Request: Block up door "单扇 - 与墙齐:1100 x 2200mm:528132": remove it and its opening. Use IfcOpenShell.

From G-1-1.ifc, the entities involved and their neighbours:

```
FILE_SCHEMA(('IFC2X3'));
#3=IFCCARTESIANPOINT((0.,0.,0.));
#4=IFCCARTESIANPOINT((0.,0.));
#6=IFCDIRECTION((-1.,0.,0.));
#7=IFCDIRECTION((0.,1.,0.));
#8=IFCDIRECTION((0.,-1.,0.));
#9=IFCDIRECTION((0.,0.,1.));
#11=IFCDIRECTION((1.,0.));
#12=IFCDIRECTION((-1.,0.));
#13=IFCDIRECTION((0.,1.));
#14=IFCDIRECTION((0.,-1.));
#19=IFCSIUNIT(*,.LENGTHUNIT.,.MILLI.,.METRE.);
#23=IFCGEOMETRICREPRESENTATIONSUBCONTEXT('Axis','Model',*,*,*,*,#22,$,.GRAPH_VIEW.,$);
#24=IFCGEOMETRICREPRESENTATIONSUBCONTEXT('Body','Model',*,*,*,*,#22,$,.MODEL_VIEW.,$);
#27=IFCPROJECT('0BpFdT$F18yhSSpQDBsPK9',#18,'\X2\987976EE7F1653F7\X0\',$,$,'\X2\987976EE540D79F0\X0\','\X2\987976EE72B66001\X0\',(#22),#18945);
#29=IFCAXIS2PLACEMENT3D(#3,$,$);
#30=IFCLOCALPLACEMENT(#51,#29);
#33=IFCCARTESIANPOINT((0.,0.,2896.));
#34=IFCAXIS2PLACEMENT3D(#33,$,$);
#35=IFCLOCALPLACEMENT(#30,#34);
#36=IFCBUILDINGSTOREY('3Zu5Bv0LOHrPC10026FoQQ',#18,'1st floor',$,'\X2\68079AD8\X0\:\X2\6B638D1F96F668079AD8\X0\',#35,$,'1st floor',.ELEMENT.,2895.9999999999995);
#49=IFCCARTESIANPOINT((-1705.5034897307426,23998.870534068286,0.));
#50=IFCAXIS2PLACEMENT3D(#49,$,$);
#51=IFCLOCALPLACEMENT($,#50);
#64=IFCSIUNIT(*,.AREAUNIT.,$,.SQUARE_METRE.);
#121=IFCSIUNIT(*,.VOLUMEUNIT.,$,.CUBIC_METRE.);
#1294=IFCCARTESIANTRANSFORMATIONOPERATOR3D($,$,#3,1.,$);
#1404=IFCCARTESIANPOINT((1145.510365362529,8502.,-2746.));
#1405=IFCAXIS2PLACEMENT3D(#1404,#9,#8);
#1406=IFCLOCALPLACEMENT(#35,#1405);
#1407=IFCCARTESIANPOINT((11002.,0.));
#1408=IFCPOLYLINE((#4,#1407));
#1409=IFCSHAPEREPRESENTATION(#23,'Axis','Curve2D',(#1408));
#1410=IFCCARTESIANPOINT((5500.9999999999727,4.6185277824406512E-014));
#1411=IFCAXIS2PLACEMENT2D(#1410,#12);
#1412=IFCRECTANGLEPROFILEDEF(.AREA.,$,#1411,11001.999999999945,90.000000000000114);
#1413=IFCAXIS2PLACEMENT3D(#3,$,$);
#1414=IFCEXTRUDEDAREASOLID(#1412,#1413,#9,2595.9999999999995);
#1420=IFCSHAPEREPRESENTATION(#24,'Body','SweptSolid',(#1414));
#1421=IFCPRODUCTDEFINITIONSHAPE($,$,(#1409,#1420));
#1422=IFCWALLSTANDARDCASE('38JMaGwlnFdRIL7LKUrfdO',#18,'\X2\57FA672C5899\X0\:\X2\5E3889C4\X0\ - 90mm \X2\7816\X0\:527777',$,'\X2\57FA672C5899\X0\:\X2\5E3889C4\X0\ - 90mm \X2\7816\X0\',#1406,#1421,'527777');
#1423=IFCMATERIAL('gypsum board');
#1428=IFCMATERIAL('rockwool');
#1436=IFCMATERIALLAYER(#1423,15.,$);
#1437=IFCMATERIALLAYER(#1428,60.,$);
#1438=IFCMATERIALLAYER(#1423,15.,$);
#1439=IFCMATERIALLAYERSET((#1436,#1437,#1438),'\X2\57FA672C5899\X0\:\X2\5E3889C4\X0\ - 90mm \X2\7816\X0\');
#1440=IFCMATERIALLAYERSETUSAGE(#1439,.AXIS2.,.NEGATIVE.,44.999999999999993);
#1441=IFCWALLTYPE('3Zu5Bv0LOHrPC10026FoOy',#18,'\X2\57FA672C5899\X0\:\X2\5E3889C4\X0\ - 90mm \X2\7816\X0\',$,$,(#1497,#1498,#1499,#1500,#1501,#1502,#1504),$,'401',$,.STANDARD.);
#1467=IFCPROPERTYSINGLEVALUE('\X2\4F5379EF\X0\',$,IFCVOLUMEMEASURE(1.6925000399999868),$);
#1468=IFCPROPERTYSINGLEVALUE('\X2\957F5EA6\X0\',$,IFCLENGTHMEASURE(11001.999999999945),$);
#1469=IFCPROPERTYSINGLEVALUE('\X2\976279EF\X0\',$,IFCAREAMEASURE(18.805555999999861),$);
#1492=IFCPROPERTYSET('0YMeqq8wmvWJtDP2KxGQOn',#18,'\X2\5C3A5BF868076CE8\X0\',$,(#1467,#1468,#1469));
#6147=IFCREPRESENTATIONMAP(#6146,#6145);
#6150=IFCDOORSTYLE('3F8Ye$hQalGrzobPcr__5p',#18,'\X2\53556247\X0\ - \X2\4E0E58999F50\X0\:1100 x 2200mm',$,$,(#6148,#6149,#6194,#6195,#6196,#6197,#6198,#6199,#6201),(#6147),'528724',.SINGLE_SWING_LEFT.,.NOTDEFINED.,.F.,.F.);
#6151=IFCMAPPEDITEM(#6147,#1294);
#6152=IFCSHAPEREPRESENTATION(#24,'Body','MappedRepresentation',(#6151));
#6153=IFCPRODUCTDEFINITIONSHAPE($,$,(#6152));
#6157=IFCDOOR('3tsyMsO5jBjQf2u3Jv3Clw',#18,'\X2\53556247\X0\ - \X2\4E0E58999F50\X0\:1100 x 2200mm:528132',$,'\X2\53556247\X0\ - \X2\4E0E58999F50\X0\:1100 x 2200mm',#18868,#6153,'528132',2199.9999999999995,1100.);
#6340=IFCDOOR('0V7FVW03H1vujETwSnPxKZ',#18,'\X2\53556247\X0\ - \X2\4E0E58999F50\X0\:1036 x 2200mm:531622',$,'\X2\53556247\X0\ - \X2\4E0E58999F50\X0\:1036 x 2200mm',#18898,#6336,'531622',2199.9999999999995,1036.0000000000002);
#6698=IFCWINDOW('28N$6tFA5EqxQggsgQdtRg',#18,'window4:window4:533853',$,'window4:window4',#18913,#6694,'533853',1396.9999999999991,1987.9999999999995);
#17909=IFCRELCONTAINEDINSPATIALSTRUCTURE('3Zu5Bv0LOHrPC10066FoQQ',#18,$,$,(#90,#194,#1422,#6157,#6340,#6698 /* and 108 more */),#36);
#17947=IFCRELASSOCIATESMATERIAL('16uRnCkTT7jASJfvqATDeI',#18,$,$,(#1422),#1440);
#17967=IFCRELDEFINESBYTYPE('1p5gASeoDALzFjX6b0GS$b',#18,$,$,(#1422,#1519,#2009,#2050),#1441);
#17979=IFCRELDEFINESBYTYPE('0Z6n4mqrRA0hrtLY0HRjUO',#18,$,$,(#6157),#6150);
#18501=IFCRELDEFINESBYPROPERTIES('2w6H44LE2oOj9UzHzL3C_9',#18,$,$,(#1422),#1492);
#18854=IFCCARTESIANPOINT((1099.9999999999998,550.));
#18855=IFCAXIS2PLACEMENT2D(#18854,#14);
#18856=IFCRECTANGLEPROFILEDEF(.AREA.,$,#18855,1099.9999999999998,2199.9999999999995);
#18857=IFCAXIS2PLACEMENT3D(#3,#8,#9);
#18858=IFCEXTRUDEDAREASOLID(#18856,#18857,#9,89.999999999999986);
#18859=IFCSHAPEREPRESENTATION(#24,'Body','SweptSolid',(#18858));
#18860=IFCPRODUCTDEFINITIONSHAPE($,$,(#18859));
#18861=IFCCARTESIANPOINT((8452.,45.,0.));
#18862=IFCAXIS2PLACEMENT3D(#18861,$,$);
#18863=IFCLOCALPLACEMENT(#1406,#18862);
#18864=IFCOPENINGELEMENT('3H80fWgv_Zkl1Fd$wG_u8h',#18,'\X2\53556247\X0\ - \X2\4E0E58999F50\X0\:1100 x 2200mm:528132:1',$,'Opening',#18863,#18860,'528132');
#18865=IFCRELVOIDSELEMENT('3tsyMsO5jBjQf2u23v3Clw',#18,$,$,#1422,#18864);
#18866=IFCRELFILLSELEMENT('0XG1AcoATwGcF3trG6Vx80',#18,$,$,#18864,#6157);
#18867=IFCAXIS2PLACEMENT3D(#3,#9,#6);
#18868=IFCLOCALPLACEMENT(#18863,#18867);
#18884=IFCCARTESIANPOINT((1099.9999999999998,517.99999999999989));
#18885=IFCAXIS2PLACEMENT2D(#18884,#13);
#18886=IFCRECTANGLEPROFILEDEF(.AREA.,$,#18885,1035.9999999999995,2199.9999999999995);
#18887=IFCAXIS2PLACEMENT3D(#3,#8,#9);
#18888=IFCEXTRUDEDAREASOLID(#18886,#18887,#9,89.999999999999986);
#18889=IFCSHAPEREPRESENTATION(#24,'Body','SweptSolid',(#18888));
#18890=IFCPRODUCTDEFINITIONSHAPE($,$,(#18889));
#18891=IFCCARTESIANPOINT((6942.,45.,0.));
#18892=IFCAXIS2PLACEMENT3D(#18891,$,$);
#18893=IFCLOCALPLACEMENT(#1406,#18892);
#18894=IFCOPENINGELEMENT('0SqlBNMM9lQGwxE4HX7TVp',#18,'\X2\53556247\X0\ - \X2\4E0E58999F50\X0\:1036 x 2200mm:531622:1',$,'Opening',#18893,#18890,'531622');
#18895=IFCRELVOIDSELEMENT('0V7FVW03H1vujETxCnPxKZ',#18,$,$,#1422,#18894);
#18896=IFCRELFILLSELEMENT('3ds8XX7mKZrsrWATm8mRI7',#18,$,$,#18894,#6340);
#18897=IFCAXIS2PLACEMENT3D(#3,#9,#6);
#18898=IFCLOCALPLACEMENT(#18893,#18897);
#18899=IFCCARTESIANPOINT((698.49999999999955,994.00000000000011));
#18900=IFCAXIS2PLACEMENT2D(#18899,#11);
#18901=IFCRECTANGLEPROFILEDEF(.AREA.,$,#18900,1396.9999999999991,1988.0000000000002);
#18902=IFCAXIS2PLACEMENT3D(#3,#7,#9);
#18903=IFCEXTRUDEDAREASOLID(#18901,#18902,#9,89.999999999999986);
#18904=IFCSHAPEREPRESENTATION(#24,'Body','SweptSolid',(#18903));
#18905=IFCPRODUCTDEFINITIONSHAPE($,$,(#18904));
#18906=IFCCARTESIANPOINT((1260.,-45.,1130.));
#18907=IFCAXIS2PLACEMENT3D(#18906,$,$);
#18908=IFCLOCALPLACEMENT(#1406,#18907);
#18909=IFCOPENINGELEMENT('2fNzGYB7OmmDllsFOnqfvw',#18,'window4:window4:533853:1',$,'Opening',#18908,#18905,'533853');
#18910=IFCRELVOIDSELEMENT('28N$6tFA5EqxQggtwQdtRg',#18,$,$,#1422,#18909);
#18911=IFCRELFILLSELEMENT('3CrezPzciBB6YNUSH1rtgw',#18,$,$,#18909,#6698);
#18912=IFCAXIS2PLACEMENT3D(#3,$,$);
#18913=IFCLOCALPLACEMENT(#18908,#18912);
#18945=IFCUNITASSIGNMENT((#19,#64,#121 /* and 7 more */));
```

```python
import ifcopenshell
import ifcopenshell.api.feature
import ifcopenshell.api.pset
import ifcopenshell.api.root
import ifcopenshell.geom
import ifcopenshell.util.element
import ifcopenshell.util.shape
import ifcopenshell.util.unit

model = ifcopenshell.open("G-1-1.ifc")
area_scale = ifcopenshell.util.unit.calculate_unit_scale(model, "AREAUNIT")
volume_scale = ifcopenshell.util.unit.calculate_unit_scale(model, "VOLUMEUNIT")
settings = ifcopenshell.geom.settings()


def volume(element):
    """Net volume in cubic metres, openings subtracted."""
    shape = ifcopenshell.geom.create_shape(settings, element)
    return ifcopenshell.util.shape.get_volume(shape.geometry)


door = model.by_id(6157)
opening = door.FillsVoids[0].RelatingOpeningElement
wall = opening.VoidsElements[0].RelatingBuildingElement
before = volume(wall)

ifcopenshell.api.root.remove_product(model, product=door)
ifcopenshell.api.feature.remove_feature(model, feature=opening)

after = volume(wall)
thickness = 0.09  # wall thickness in metres

# Update the wall's stored quantities.
pset = model.by_id(ifcopenshell.util.element.get_pset(wall, "尺寸标注", should_inherit=False)["id"])
ifcopenshell.api.pset.edit_pset(model, pset=pset, properties={
    "体积": model.create_entity("IfcVolumeMeasure", after / volume_scale),
    "面积": model.create_entity("IfcAreaMeasure", after / thickness / area_scale),
})

print(f"wall volume {before:.3f} -> {after:.3f} m3")

model.write("G-1-1-out.ifc")
```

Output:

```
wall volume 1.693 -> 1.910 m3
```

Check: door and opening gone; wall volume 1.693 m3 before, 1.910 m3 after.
